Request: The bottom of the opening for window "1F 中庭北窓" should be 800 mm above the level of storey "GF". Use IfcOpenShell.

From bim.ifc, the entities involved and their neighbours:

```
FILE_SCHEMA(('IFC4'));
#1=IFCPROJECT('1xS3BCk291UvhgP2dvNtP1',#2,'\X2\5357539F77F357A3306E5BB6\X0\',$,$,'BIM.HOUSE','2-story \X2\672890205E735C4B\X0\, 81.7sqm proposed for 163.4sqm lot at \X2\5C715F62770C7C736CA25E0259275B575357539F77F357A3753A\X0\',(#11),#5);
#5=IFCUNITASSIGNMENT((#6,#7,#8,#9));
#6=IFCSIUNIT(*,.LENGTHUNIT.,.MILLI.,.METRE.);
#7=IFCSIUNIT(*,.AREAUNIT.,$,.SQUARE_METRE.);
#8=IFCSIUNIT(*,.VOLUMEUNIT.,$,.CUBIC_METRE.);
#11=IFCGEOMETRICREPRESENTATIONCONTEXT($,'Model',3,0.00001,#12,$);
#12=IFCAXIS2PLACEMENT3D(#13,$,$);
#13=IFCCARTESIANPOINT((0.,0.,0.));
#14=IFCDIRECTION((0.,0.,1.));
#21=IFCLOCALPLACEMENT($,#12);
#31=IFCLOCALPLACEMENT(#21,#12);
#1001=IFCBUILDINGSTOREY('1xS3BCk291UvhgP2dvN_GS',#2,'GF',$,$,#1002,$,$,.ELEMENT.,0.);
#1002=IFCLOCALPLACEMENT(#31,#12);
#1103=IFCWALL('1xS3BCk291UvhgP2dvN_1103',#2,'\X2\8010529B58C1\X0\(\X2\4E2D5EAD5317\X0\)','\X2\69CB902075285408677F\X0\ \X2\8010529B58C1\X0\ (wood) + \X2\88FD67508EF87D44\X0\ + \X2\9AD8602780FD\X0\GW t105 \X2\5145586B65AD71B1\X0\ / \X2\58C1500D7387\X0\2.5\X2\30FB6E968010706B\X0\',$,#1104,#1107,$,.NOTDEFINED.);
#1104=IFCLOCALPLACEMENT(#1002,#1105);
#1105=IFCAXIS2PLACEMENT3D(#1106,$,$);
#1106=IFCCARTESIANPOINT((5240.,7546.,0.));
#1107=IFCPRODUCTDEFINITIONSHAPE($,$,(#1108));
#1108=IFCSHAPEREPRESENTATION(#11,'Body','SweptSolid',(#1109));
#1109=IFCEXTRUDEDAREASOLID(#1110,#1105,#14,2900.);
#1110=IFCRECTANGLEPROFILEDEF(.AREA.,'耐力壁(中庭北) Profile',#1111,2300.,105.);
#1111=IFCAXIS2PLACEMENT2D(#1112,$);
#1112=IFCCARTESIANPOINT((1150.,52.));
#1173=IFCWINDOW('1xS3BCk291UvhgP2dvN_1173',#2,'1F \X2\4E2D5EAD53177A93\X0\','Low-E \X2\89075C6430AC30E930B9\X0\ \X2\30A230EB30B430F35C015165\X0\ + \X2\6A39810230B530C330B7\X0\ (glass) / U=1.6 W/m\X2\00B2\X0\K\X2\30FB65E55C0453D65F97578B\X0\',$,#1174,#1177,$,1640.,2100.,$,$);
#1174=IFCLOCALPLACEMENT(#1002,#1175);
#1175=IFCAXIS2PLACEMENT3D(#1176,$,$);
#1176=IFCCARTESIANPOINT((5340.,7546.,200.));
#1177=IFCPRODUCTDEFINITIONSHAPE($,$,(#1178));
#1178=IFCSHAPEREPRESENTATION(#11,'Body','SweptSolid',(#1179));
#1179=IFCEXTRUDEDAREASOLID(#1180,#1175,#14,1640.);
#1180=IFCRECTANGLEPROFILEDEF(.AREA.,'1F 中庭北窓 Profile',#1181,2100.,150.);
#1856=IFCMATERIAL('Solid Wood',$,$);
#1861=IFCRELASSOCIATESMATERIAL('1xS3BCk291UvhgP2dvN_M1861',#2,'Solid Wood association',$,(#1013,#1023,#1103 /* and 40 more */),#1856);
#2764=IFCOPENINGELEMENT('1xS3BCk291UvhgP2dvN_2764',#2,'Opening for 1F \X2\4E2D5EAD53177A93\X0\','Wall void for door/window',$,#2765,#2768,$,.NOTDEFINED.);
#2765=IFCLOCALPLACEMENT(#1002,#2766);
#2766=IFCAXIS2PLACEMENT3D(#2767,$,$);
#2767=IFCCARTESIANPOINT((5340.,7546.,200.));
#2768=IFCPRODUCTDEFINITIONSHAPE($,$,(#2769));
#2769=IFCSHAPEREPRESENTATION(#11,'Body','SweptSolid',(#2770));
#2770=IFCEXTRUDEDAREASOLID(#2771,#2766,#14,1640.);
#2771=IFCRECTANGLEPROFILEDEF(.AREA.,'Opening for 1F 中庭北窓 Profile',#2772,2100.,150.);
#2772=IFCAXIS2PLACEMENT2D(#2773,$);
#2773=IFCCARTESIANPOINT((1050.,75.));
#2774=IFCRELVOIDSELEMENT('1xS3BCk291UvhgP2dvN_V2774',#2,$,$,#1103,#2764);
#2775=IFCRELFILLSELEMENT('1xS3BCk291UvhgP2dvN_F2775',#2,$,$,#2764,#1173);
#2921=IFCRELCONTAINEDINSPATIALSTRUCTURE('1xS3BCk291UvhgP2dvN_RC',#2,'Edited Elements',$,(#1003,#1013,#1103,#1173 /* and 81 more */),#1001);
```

```python
import numpy as np
import ifcopenshell
import ifcopenshell.api.geometry
import ifcopenshell.geom
import ifcopenshell.util.element
import ifcopenshell.util.placement
import ifcopenshell.util.shape
import ifcopenshell.util.unit

model = ifcopenshell.open("bim.ifc")
unit_scale = ifcopenshell.util.unit.calculate_unit_scale(model)

window = model.by_guid("1xS3BCk291UvhgP2dvN_1173")
opening = window.FillsVoids[0].RelatingOpeningElement
storey = ifcopenshell.util.element.get_container(window, ifc_class="IfcBuildingStorey")
level = ifcopenshell.util.placement.get_local_placement(storey.ObjectPlacement)[2, 3]

# The opening's origin need not be at the sill, so measure its lowest point.
shape = ifcopenshell.geom.create_shape(ifcopenshell.geom.settings(), opening)
bottom = ifcopenshell.util.shape.get_shape_bottom_elevation(shape, shape.geometry) / unit_scale
dz = level + 0.8 / unit_scale - bottom

shift = np.array([0.0, 0.0, dz])
# The window is not placed relative to its opening, so move both.
for product in (opening, window):
    matrix = ifcopenshell.util.placement.get_local_placement(product.ObjectPlacement)
    matrix[:3, 3] += shift
    ifcopenshell.api.geometry.edit_object_placement(model, product=product, matrix=matrix, is_si=False)

print(f"moved by {dz * unit_scale:+.3f} m")

model.write("bim_rev.ifc")
```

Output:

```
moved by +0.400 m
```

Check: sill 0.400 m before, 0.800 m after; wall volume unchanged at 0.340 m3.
